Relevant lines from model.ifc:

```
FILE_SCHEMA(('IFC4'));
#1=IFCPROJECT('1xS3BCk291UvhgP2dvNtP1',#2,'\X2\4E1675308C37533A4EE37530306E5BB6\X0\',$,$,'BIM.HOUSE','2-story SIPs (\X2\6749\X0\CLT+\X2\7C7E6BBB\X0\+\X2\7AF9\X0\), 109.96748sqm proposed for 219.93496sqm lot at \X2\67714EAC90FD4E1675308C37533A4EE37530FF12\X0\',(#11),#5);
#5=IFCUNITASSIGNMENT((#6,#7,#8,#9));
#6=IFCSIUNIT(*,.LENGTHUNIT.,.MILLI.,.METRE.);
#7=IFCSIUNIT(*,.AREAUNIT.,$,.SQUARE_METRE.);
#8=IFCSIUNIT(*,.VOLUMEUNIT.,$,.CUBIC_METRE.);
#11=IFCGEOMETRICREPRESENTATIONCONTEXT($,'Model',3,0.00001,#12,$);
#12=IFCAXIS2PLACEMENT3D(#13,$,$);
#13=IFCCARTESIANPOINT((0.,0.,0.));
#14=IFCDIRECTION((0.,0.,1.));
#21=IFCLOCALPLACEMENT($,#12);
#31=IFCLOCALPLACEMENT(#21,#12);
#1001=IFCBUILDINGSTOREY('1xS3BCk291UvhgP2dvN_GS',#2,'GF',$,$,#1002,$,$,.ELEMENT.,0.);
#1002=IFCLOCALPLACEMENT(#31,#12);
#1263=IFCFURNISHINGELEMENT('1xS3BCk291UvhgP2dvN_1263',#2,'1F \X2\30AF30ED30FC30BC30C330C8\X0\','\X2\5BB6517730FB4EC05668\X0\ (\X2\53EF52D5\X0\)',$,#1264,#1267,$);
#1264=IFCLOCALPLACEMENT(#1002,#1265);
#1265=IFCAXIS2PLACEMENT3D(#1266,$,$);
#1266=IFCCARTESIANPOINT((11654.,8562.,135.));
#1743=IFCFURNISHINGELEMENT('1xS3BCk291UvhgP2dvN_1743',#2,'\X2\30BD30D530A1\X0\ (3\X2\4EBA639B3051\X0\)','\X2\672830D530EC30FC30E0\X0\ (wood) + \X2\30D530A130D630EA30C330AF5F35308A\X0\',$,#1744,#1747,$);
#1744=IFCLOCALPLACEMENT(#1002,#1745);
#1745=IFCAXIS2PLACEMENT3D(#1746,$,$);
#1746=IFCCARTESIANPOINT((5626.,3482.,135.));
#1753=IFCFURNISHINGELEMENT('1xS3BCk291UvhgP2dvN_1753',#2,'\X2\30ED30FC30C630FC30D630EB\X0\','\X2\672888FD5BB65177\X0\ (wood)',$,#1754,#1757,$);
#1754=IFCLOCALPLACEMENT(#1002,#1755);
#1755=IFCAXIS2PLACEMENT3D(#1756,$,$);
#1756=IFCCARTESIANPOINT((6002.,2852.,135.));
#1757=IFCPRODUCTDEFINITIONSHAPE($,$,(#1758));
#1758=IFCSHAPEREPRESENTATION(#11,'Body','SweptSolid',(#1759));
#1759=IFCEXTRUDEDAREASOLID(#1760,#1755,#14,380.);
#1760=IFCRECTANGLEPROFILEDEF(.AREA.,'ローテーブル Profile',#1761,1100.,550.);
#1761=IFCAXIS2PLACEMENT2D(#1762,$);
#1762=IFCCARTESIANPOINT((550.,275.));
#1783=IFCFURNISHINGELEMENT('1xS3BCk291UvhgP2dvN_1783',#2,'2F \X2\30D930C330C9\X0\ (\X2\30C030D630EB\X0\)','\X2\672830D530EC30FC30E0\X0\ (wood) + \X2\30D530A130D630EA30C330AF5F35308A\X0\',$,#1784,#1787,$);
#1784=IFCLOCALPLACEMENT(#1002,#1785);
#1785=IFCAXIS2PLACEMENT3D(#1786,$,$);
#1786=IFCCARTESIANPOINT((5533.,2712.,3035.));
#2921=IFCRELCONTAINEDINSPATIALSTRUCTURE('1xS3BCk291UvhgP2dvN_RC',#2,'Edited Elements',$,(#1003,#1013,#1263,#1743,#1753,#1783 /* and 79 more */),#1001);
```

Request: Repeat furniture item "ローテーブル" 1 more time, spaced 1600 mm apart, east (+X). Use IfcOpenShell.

```python
import numpy as np
import ifcopenshell
import ifcopenshell.api.geometry
import ifcopenshell.api.root
import ifcopenshell.util.element
import ifcopenshell.util.placement
import ifcopenshell.util.unit

model = ifcopenshell.open("model.ifc")
unit_scale = ifcopenshell.util.unit.calculate_unit_scale(model)


def reuse_history(source, copy):
    """copy_class also copies each property set's owner history, people and application; keep the originals."""
    for rel in copy.IsDefinedBy:
        if rel.is_a("IfcRelDefinesByProperties") and (history := rel.RelatingPropertyDefinition.OwnerHistory):
            rel.RelatingPropertyDefinition.OwnerHistory = source.OwnerHistory
            ifcopenshell.util.element.remove_deep2(model, history)


source = model.by_guid("1xS3BCk291UvhgP2dvN_1753")
base = ifcopenshell.util.placement.get_local_placement(source.ObjectPlacement)
step = np.array([1.0, 0.0, 0.0]) * 1.6 / unit_scale

for i in range(1, 2):
    copy = ifcopenshell.api.root.copy_class(model, product=source)
    copy.Representation = ifcopenshell.util.element.copy_deep(
        model, source.Representation, exclude=["IfcGeometricRepresentationContext", "IfcRepresentationMap"]
    )
    reuse_history(source, copy)
    matrix = base.copy()
    matrix[:3, 3] += i * step
    print("added at", matrix[:3, 3].round(3) + 0.0)
    ifcopenshell.api.geometry.edit_object_placement(model, product=copy, matrix=matrix, is_si=False)

model.write("model_v2.ifc")
```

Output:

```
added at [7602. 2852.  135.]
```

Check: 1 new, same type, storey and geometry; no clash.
